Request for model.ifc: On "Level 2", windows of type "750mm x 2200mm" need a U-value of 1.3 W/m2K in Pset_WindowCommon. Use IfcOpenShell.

First a look at what the model holds.

```python
import ifcopenshell
import ifcopenshell.util.element

model = ifcopenshell.open("model.ifc")
print(model.schema)
storey = next(s for s in model.by_type("IfcBuildingStorey") if s.Name == "Level 2")
windows = [e for e in ifcopenshell.util.element.get_decomposition(storey) if e.is_a("IfcWindow")]
seen = {}
for e in windows:
    element_type = ifcopenshell.util.element.get_type(e)
    key = (element_type.Name if element_type != e and element_type else None, ifcopenshell.util.element.get_pset(e, "Pset_WindowCommon", "ThermalTransmittance"))
    seen[key] = seen.get(key, 0) + 1
for (name, value), count in sorted(seen.items(), key=str):
    print(count, "x", name, "|", value)
```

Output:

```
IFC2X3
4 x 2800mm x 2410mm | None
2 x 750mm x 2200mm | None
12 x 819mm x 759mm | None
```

```python
import ifcopenshell
import ifcopenshell.api.pset
import ifcopenshell.util.element

model = ifcopenshell.open("model.ifc")

storey = next(s for s in model.by_type("IfcBuildingStorey") if s.Name == "Level 2")
windows = [e for e in ifcopenshell.util.element.get_decomposition(storey) if e.is_a("IfcWindow")]

count = 0
for e in windows:
    element_type = ifcopenshell.util.element.get_type(e)
    if element_type in (None, e) or element_type.Name != "750mm x 2200mm":
        continue
    # add_pset returns the element's existing set when there is one.
    pset = ifcopenshell.api.pset.add_pset(model, product=e, name="Pset_WindowCommon")
    ifcopenshell.api.pset.edit_pset(model, pset=pset, properties={"ThermalTransmittance": 1.3})
    count += 1

print(count, "windows updated")

model.write("model-out.ifc")
```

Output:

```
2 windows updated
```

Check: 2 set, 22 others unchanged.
